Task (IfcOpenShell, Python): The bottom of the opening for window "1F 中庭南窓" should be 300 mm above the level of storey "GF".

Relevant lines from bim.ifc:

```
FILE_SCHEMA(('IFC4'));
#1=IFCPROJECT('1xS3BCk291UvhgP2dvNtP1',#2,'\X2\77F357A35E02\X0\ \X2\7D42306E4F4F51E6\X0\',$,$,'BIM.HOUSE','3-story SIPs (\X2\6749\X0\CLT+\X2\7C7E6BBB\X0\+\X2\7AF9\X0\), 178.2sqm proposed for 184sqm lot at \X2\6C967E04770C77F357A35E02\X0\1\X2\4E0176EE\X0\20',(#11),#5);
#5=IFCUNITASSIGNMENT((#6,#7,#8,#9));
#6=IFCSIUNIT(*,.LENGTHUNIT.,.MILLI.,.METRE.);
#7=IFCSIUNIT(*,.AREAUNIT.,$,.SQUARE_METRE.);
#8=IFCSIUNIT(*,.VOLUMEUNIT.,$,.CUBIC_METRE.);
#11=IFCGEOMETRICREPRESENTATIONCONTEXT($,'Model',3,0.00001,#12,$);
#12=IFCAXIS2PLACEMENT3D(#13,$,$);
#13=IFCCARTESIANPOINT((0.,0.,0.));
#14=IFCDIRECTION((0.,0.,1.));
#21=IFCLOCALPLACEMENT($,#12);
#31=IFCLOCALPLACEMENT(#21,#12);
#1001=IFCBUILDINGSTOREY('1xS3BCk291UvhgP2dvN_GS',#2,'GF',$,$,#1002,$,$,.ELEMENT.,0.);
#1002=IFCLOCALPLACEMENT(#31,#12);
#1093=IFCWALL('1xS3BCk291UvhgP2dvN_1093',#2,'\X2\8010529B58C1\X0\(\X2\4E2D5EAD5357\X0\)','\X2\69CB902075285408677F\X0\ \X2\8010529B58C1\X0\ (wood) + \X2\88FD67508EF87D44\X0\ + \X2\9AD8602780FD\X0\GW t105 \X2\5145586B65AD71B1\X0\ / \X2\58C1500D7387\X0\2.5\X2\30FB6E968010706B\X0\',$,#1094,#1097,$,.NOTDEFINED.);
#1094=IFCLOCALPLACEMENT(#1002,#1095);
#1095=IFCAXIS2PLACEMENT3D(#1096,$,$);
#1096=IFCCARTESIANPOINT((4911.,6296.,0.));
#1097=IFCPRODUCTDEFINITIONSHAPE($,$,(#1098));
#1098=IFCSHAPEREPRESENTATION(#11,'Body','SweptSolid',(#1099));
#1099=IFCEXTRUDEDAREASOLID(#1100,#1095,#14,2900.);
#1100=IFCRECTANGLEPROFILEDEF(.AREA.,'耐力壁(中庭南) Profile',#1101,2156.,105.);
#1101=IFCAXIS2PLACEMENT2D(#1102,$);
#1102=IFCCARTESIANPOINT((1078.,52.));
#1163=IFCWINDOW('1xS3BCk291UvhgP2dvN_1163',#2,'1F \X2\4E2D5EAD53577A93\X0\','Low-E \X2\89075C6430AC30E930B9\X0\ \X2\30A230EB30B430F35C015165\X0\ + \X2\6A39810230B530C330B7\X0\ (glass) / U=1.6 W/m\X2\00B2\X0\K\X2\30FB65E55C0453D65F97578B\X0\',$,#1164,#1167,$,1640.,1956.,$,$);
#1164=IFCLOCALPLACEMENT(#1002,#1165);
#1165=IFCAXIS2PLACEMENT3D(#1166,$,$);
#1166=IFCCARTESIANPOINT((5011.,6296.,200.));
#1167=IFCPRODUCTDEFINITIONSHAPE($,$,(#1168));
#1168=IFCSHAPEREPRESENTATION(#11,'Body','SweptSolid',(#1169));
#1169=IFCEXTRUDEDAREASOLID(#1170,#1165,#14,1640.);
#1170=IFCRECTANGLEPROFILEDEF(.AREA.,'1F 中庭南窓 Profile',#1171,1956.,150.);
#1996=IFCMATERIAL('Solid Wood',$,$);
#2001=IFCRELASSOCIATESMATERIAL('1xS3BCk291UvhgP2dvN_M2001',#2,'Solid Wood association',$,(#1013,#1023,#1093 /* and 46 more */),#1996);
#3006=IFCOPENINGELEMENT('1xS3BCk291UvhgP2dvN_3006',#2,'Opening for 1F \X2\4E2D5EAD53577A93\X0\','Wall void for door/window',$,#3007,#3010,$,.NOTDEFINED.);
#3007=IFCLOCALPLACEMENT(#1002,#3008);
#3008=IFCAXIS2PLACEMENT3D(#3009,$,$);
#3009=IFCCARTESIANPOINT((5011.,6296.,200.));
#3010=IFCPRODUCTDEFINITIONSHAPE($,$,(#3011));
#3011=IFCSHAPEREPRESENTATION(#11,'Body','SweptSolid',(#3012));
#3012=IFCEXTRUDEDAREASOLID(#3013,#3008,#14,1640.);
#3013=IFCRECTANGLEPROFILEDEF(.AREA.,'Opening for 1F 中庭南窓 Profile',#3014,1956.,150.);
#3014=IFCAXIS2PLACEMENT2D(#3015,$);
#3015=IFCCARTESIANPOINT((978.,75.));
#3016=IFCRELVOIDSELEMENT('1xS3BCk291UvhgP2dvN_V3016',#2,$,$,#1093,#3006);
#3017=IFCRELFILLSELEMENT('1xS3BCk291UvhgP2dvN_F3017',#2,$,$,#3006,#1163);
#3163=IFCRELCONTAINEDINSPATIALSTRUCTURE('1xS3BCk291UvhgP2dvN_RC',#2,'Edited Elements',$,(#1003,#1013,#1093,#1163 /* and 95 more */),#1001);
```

```python
import numpy as np
import ifcopenshell
import ifcopenshell.api.geometry
import ifcopenshell.geom
import ifcopenshell.util.element
import ifcopenshell.util.placement
import ifcopenshell.util.shape
import ifcopenshell.util.unit

model = ifcopenshell.open("bim.ifc")
unit_scale = ifcopenshell.util.unit.calculate_unit_scale(model)

window = model.by_id(1163)
opening = window.FillsVoids[0].RelatingOpeningElement
storey = ifcopenshell.util.element.get_container(window, ifc_class="IfcBuildingStorey")
level = ifcopenshell.util.placement.get_local_placement(storey.ObjectPlacement)[2, 3]

# The opening's origin need not be at the sill, so measure its lowest point.
shape = ifcopenshell.geom.create_shape(ifcopenshell.geom.settings(), opening)
bottom = ifcopenshell.util.shape.get_shape_bottom_elevation(shape, shape.geometry) / unit_scale
dz = level + 300.0 - bottom

shift = np.array([0.0, 0.0, dz])
# The window is not placed relative to its opening, so move both.
for product in (opening, window):
    matrix = ifcopenshell.util.placement.get_local_placement(product.ObjectPlacement)
    matrix[:3, 3] += shift
    ifcopenshell.api.geometry.edit_object_placement(model, product=product, matrix=matrix, is_si=False)

print(f"moved by {dz * unit_scale:+.3f} m")

model.write("bim_edited.ifc")
```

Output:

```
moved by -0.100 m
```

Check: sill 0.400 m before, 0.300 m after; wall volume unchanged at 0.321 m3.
